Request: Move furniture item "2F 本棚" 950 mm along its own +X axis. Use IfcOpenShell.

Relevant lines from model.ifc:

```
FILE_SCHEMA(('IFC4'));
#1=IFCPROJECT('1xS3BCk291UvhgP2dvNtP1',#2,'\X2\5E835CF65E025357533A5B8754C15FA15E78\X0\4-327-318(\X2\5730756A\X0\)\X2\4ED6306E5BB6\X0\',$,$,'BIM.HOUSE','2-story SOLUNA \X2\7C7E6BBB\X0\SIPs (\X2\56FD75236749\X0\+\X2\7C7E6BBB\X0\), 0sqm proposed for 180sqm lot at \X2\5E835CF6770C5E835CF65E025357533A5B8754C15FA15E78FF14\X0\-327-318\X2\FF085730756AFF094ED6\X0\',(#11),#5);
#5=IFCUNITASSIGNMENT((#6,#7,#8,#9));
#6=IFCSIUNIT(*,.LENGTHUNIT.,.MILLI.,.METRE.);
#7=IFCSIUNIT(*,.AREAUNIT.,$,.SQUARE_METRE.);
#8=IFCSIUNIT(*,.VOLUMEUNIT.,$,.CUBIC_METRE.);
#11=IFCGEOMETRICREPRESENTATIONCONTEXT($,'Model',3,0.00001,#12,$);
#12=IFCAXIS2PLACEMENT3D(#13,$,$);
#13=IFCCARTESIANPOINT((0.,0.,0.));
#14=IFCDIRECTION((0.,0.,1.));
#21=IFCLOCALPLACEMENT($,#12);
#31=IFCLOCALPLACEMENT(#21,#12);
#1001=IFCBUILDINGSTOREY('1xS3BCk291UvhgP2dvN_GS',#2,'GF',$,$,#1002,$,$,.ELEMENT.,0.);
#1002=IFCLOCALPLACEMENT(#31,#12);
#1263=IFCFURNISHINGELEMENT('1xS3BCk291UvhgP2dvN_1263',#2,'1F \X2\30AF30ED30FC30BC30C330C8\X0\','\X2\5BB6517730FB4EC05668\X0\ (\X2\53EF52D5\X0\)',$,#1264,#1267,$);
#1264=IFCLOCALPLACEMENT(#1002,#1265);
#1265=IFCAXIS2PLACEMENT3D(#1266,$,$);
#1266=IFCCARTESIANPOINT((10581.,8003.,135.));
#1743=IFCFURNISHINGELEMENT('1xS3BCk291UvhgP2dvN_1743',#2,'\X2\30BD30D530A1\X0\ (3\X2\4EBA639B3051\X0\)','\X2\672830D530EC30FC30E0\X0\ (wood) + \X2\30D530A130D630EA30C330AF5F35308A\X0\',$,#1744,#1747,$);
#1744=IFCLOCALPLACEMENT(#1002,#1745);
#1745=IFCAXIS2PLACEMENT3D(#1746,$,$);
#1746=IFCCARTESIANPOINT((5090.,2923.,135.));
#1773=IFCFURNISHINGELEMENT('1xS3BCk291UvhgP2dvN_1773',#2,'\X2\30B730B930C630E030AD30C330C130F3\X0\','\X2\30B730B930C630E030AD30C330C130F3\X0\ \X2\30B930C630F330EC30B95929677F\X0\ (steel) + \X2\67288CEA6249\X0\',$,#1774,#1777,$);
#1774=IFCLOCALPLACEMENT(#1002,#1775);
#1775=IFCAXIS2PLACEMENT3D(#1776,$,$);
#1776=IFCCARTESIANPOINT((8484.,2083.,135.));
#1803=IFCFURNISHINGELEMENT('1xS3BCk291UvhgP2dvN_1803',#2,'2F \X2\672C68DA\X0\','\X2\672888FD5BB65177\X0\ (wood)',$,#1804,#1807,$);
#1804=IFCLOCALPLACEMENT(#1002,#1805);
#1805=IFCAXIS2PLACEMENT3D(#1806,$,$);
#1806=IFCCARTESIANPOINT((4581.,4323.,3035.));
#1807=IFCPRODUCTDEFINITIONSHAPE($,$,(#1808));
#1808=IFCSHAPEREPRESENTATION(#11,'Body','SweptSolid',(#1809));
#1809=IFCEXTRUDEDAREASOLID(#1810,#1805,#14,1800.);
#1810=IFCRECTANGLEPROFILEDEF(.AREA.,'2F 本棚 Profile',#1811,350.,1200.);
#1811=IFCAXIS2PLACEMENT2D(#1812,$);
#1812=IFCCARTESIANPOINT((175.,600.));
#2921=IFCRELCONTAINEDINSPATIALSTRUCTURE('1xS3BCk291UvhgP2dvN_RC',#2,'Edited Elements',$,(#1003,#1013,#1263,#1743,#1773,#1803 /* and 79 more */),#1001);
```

```python
import ifcopenshell
import ifcopenshell.api.geometry
import ifcopenshell.util.placement
import ifcopenshell.util.unit

model = ifcopenshell.open("model.ifc")
unit_scale = ifcopenshell.util.unit.calculate_unit_scale(model)

item = model.by_guid("1xS3BCk291UvhgP2dvN_1803")
matrix = ifcopenshell.util.placement.get_local_placement(item.ObjectPlacement)
matrix[:3, 3] += matrix[:3, 0] * 0.95 / unit_scale
ifcopenshell.api.geometry.edit_object_placement(model, product=item, matrix=matrix, is_si=False)

print(ifcopenshell.util.placement.get_local_placement(item.ObjectPlacement).round(3) + 0.0)

model.write("model_v2.ifc")
```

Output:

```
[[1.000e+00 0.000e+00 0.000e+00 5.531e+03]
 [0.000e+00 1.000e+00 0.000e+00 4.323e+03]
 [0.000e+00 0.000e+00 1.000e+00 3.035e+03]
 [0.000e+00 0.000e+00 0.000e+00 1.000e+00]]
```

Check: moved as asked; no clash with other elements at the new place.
